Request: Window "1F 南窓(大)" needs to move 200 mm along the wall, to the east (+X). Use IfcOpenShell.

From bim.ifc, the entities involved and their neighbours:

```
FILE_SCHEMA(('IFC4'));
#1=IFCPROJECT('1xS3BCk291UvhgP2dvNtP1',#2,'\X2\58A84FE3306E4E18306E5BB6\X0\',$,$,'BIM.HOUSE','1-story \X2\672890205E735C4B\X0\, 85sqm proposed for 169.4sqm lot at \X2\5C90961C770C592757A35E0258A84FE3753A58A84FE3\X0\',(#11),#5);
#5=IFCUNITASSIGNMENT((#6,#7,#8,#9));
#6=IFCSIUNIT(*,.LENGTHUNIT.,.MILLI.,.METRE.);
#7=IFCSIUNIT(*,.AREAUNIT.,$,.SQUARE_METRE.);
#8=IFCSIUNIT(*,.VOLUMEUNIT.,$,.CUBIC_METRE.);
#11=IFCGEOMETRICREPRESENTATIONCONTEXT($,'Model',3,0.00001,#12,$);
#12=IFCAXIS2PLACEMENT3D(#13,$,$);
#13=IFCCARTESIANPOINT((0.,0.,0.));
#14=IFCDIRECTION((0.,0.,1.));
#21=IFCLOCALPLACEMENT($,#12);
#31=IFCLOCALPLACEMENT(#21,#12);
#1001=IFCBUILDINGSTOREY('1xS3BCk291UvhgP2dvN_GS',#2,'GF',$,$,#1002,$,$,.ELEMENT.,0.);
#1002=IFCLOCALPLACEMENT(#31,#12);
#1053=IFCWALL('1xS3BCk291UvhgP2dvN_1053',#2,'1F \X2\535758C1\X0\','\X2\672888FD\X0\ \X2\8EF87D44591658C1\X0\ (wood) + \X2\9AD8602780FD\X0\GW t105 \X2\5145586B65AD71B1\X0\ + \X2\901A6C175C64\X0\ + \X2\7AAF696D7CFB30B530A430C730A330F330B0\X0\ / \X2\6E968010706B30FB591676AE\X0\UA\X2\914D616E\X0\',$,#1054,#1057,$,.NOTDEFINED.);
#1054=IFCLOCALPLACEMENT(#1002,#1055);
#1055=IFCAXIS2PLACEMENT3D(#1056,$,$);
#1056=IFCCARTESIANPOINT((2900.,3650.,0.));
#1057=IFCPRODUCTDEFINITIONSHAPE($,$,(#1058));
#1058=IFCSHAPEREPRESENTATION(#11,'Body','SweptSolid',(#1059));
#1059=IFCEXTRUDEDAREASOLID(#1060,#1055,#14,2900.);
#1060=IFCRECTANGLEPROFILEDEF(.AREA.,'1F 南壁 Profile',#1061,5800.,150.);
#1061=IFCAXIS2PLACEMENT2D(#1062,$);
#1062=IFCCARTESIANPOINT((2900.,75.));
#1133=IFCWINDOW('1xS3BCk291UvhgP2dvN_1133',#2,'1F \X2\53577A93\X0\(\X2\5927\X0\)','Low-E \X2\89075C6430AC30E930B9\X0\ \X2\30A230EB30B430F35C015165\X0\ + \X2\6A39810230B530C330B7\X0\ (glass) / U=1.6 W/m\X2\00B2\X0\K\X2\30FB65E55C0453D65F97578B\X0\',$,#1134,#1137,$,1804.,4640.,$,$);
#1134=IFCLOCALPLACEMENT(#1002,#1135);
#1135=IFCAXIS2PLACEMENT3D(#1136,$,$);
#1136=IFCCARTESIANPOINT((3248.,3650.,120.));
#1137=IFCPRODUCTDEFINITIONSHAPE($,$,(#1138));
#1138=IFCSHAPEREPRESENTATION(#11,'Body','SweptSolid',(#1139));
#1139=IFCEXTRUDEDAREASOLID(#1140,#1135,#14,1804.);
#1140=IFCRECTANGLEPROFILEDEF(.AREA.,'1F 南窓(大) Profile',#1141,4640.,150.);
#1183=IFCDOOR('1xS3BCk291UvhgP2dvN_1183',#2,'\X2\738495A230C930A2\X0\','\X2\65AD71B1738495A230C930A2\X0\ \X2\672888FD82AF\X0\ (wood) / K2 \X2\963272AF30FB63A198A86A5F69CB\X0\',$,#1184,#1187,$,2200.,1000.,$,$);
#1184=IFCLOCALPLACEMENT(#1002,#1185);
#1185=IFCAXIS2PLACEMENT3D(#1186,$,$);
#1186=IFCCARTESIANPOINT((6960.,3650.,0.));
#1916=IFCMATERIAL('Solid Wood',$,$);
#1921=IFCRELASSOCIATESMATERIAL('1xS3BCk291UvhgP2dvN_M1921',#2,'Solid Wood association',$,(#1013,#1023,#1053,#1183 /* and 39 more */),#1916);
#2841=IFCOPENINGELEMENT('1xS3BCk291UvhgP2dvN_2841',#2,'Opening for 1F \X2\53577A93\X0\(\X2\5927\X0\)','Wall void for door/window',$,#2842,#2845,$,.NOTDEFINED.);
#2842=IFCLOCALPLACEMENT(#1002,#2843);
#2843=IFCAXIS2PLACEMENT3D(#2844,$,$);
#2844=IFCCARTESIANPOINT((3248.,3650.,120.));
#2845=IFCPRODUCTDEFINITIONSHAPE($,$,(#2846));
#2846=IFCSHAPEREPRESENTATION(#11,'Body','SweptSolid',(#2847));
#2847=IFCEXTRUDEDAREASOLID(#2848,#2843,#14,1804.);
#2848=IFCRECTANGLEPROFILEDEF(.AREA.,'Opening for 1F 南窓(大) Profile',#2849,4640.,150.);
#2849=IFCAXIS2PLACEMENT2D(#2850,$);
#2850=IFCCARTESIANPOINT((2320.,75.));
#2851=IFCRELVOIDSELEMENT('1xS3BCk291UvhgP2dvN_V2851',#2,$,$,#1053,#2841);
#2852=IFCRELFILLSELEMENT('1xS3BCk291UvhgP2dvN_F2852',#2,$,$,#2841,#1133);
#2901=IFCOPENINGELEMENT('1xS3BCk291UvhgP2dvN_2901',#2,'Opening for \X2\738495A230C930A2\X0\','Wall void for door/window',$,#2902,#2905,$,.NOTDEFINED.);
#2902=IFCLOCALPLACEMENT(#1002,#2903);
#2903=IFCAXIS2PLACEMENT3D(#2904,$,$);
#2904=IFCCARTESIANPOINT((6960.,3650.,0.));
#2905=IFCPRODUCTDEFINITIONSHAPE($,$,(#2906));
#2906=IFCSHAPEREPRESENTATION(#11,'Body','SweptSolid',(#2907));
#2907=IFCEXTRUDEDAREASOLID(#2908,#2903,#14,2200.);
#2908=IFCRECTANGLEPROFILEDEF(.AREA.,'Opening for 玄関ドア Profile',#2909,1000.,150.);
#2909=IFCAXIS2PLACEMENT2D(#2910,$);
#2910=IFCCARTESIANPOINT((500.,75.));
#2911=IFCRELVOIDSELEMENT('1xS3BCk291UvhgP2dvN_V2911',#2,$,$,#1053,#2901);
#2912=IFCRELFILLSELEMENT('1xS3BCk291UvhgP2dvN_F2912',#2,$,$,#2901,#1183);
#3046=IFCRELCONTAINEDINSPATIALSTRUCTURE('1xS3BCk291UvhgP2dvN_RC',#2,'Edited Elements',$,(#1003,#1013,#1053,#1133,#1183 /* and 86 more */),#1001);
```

```python
import ifcopenshell
import ifcopenshell.api.geometry
import ifcopenshell.util.placement
import ifcopenshell.util.unit

model = ifcopenshell.open("bim.ifc")
unit_scale = ifcopenshell.util.unit.calculate_unit_scale(model)

window = model.by_guid("1xS3BCk291UvhgP2dvN_1133")
opening = window.FillsVoids[0].RelatingOpeningElement
wall = opening.VoidsElements[0].RelatingBuildingElement

wall_matrix = ifcopenshell.util.placement.get_local_placement(wall.ObjectPlacement)
shift = wall_matrix[:3, 0] * 0.2 / unit_scale
before = ifcopenshell.util.placement.get_local_placement(window.ObjectPlacement)[:3, 3].copy()

# The window is not placed relative to its opening, so move both.
for product in (opening, window):
    matrix = ifcopenshell.util.placement.get_local_placement(product.ObjectPlacement)
    matrix[:3, 3] += shift
    ifcopenshell.api.geometry.edit_object_placement(model, product=product, matrix=matrix, is_si=False)

after = ifcopenshell.util.placement.get_local_placement(window.ObjectPlacement)[:3, 3]
print("window moved by", (after - before).round(3) + 0.0)

model.write("bim_edited.ifc")
```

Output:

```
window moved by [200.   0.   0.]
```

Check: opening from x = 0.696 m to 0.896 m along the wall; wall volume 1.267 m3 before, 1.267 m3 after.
